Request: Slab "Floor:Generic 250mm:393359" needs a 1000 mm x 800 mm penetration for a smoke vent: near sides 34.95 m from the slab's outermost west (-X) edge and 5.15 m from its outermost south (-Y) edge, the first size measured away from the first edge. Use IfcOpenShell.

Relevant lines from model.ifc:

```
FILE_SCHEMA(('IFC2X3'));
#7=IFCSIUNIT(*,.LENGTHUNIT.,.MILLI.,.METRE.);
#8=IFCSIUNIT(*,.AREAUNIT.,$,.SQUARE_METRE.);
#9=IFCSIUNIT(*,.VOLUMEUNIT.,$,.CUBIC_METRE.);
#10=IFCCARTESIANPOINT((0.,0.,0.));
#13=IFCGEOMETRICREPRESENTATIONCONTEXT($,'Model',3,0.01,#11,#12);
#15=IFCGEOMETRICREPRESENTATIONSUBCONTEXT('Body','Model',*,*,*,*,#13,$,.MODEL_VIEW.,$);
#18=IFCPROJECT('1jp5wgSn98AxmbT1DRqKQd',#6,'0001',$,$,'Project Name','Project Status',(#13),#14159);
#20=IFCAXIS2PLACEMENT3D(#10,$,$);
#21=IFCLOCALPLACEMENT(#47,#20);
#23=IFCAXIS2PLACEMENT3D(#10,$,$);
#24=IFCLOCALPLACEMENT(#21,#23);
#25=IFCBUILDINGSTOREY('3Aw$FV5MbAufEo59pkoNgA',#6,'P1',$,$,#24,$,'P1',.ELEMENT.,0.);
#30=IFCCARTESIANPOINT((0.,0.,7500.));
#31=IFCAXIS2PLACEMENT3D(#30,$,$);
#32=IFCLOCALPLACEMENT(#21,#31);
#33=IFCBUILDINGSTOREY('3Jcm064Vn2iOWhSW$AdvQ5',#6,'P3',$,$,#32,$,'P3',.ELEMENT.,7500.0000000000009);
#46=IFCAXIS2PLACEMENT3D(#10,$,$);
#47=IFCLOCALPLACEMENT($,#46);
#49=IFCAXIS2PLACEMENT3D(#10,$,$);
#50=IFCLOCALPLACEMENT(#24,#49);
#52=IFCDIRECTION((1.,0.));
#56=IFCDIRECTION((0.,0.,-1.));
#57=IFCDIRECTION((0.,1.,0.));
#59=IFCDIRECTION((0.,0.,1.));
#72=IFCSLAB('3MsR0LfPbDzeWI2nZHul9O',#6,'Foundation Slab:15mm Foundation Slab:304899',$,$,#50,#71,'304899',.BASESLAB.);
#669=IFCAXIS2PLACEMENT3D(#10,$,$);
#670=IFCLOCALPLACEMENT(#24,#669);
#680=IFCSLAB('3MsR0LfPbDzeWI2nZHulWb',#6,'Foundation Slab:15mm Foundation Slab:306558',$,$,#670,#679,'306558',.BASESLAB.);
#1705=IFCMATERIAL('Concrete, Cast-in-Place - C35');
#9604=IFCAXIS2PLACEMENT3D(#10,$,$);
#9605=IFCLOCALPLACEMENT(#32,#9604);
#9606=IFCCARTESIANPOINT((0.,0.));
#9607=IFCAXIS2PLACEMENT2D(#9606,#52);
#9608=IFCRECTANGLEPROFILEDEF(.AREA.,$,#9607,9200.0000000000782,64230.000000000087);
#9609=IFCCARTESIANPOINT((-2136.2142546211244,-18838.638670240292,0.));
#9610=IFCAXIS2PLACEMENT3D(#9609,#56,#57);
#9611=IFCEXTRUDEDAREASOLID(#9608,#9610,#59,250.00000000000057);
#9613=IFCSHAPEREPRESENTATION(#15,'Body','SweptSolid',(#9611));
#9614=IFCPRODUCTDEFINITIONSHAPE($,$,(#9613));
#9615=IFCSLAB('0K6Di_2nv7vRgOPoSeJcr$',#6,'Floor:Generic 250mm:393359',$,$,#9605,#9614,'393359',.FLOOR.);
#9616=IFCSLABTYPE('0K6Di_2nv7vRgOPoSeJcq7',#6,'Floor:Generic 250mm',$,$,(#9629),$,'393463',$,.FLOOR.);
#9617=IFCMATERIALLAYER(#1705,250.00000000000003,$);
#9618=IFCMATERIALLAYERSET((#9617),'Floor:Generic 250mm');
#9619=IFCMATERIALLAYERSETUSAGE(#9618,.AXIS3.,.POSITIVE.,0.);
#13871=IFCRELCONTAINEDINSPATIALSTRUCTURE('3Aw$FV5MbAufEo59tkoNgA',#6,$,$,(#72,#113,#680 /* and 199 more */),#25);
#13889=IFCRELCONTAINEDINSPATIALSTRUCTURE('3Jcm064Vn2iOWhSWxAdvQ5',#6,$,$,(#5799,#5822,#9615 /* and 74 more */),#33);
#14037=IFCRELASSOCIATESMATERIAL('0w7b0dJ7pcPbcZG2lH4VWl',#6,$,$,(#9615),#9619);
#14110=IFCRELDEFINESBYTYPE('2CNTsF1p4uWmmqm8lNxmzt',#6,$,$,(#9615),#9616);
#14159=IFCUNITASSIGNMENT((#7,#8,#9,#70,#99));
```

```python
import numpy as np
import ifcopenshell
import ifcopenshell.api.feature
import ifcopenshell.api.geometry
import ifcopenshell.api.root
import ifcopenshell.geom
import ifcopenshell.util.placement
import ifcopenshell.util.representation
import ifcopenshell.util.shape
import ifcopenshell.util.unit

model = ifcopenshell.open("model.ifc")
unit_scale = ifcopenshell.util.unit.calculate_unit_scale(model)
settings = ifcopenshell.geom.settings()


def volume(element):
    """Net volume in cubic metres, openings subtracted."""
    shape = ifcopenshell.geom.create_shape(settings, element)
    return ifcopenshell.util.shape.get_volume(shape.geometry)


slab = model.by_id(9615)
before = volume(slab)

# Extent in the slab's own axes, in metres. The edges named are its -X and -Y sides.
slab_shape = ifcopenshell.geom.create_shape(settings, slab)
vertices = ifcopenshell.util.shape.get_vertices(slab_shape.geometry)
x_min, y_min, bottom = vertices.min(axis=0)
top = vertices[:, 2].max()

opening = ifcopenshell.api.root.create_entity(model, ifc_class="IfcOpeningElement", name="Smoke vent opening")
context = ifcopenshell.util.representation.get_context(model, "Model", "Body", "MODEL_VIEW")
width, depth = 1, 0.8
outline = [(0.0, 0.0), (width, 0.0), (width, depth), (0.0, depth), (0.0, 0.0)]
# Overshoot both faces by 50 mm so the cut is clean.
shape = ifcopenshell.api.geometry.add_slab_representation(
    model, context=context, depth=top - bottom + 0.1, polyline=outline
)
ifcopenshell.api.geometry.assign_representation(model, product=opening, representation=shape)

matrix = ifcopenshell.util.placement.get_local_placement(slab.ObjectPlacement)
matrix[:, 3] = matrix @ np.append(np.array([x_min + 34.95, y_min + 5.15, bottom - 0.05]) / unit_scale, 1.0)
ifcopenshell.api.geometry.edit_object_placement(model, product=opening, matrix=matrix, is_si=False)
ifcopenshell.api.feature.add_feature(model, feature=opening, element=slab)

after = volume(slab)

print(f"slab volume {before:.3f} -> {after:.3f} m3")

model.write("model_updated.ifc")
```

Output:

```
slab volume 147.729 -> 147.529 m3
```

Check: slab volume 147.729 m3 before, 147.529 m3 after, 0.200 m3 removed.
